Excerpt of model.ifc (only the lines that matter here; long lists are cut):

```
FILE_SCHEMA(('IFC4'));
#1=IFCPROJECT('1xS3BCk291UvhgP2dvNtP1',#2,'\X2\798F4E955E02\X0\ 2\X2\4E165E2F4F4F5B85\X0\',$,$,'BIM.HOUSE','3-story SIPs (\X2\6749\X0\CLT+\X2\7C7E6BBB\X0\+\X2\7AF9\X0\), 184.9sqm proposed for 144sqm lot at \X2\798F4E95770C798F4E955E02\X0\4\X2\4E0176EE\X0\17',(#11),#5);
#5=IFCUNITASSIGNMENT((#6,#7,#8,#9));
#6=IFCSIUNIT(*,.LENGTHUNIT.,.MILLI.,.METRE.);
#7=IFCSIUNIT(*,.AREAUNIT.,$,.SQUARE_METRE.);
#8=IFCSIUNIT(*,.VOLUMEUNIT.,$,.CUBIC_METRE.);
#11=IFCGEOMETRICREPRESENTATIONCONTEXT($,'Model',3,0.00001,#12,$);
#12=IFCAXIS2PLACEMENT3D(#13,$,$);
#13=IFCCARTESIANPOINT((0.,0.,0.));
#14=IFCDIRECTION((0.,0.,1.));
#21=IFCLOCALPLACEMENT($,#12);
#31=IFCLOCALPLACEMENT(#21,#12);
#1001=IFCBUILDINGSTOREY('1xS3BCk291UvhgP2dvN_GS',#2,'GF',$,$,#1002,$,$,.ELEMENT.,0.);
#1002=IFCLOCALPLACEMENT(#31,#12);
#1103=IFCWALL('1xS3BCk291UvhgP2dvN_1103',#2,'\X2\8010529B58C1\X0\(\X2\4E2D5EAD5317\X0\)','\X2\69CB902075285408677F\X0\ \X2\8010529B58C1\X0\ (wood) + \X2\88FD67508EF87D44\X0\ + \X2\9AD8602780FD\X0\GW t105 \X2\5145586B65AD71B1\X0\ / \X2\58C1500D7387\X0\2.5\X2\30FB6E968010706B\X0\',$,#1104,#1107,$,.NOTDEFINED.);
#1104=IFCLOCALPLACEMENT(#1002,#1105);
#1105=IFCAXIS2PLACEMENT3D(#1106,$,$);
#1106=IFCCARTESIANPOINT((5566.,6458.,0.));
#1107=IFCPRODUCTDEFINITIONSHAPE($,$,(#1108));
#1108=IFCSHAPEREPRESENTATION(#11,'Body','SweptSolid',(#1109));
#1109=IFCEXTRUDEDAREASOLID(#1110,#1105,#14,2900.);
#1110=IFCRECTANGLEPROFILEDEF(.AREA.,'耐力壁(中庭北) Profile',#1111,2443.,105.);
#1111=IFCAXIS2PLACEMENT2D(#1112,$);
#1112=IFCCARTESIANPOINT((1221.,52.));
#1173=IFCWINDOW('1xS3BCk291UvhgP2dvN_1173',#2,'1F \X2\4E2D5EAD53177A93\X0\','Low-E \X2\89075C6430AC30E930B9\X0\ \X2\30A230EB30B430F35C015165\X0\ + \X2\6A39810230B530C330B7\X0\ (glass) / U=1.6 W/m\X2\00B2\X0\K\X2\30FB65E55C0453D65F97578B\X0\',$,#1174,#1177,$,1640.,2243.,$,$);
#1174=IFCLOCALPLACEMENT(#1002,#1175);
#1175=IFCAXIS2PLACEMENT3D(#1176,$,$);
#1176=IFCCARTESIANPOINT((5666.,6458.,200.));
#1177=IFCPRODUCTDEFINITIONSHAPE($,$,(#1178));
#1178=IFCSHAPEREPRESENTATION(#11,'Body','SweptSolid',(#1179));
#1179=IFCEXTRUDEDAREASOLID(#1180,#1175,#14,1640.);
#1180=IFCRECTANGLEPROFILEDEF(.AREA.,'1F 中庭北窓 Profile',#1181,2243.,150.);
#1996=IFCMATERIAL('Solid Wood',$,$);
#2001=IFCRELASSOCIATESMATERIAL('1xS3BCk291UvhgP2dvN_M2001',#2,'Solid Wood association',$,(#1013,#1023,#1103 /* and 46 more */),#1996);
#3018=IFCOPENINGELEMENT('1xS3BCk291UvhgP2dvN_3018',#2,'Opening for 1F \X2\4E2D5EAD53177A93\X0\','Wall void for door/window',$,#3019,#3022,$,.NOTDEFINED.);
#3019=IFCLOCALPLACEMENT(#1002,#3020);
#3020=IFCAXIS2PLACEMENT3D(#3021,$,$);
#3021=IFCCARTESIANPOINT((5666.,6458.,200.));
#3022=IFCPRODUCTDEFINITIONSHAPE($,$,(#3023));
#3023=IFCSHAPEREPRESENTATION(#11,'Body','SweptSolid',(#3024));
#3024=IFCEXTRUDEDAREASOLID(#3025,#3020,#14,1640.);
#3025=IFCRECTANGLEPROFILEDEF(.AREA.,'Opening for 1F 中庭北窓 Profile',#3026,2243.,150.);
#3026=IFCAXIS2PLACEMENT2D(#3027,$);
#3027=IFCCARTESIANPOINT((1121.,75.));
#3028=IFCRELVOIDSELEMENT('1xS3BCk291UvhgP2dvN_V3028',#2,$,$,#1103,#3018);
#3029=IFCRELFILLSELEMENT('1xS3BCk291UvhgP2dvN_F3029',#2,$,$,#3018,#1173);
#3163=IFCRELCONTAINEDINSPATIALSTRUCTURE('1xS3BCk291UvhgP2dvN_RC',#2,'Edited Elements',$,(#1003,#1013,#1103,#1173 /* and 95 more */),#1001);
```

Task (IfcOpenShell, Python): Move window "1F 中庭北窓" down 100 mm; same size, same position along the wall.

```python
import numpy as np
import ifcopenshell
import ifcopenshell.api.geometry
import ifcopenshell.util.placement
import ifcopenshell.util.unit

model = ifcopenshell.open("model.ifc")
unit_scale = ifcopenshell.util.unit.calculate_unit_scale(model)

window = model.by_id(1173)
opening = window.FillsVoids[0].RelatingOpeningElement
dz = -0.1 / unit_scale

shift = np.array([0.0, 0.0, dz])
# The window is not placed relative to its opening, so move both.
for product in (opening, window):
    matrix = ifcopenshell.util.placement.get_local_placement(product.ObjectPlacement)
    matrix[:3, 3] += shift
    ifcopenshell.api.geometry.edit_object_placement(model, product=product, matrix=matrix, is_si=False)

print(f"moved by {dz * unit_scale:+.3f} m")

model.write("model_rev.ifc")
```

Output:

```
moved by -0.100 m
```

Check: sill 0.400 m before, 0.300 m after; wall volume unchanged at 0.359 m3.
